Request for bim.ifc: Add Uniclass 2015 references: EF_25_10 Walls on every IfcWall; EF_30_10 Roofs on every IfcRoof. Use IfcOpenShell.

First a look at what the model holds.

```python
import ifcopenshell

model = ifcopenshell.open("bim.ifc")
print(model.schema)
print("classifications:", [c.Name for c in model.by_type("IfcClassification")])
for ifc_class in ("IfcDoor", "IfcRoof", "IfcStair", "IfcWall", "IfcWindow"):
    print(ifc_class, len(model.by_type(ifc_class)))
```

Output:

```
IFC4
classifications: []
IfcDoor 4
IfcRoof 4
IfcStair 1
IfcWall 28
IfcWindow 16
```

```python
import ifcopenshell
import ifcopenshell.api.classification

model = ifcopenshell.open("bim.ifc")

system = ifcopenshell.api.classification.add_classification(model, classification="Uniclass 2015")

codes = {
    "IfcWall": ("EF_25_10", "Walls"),
    "IfcRoof": ("EF_30_10", "Roofs"),
}
for ifc_class, (code, name) in codes.items():
    products = model.by_type(ifc_class)
    ifcopenshell.api.classification.add_reference(
        model, products=products, classification=system, identification=code, name=name
    )
    print(code, len(products))

model.write("bim_updated.ifc")
```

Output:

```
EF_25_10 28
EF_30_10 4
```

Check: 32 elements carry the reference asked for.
